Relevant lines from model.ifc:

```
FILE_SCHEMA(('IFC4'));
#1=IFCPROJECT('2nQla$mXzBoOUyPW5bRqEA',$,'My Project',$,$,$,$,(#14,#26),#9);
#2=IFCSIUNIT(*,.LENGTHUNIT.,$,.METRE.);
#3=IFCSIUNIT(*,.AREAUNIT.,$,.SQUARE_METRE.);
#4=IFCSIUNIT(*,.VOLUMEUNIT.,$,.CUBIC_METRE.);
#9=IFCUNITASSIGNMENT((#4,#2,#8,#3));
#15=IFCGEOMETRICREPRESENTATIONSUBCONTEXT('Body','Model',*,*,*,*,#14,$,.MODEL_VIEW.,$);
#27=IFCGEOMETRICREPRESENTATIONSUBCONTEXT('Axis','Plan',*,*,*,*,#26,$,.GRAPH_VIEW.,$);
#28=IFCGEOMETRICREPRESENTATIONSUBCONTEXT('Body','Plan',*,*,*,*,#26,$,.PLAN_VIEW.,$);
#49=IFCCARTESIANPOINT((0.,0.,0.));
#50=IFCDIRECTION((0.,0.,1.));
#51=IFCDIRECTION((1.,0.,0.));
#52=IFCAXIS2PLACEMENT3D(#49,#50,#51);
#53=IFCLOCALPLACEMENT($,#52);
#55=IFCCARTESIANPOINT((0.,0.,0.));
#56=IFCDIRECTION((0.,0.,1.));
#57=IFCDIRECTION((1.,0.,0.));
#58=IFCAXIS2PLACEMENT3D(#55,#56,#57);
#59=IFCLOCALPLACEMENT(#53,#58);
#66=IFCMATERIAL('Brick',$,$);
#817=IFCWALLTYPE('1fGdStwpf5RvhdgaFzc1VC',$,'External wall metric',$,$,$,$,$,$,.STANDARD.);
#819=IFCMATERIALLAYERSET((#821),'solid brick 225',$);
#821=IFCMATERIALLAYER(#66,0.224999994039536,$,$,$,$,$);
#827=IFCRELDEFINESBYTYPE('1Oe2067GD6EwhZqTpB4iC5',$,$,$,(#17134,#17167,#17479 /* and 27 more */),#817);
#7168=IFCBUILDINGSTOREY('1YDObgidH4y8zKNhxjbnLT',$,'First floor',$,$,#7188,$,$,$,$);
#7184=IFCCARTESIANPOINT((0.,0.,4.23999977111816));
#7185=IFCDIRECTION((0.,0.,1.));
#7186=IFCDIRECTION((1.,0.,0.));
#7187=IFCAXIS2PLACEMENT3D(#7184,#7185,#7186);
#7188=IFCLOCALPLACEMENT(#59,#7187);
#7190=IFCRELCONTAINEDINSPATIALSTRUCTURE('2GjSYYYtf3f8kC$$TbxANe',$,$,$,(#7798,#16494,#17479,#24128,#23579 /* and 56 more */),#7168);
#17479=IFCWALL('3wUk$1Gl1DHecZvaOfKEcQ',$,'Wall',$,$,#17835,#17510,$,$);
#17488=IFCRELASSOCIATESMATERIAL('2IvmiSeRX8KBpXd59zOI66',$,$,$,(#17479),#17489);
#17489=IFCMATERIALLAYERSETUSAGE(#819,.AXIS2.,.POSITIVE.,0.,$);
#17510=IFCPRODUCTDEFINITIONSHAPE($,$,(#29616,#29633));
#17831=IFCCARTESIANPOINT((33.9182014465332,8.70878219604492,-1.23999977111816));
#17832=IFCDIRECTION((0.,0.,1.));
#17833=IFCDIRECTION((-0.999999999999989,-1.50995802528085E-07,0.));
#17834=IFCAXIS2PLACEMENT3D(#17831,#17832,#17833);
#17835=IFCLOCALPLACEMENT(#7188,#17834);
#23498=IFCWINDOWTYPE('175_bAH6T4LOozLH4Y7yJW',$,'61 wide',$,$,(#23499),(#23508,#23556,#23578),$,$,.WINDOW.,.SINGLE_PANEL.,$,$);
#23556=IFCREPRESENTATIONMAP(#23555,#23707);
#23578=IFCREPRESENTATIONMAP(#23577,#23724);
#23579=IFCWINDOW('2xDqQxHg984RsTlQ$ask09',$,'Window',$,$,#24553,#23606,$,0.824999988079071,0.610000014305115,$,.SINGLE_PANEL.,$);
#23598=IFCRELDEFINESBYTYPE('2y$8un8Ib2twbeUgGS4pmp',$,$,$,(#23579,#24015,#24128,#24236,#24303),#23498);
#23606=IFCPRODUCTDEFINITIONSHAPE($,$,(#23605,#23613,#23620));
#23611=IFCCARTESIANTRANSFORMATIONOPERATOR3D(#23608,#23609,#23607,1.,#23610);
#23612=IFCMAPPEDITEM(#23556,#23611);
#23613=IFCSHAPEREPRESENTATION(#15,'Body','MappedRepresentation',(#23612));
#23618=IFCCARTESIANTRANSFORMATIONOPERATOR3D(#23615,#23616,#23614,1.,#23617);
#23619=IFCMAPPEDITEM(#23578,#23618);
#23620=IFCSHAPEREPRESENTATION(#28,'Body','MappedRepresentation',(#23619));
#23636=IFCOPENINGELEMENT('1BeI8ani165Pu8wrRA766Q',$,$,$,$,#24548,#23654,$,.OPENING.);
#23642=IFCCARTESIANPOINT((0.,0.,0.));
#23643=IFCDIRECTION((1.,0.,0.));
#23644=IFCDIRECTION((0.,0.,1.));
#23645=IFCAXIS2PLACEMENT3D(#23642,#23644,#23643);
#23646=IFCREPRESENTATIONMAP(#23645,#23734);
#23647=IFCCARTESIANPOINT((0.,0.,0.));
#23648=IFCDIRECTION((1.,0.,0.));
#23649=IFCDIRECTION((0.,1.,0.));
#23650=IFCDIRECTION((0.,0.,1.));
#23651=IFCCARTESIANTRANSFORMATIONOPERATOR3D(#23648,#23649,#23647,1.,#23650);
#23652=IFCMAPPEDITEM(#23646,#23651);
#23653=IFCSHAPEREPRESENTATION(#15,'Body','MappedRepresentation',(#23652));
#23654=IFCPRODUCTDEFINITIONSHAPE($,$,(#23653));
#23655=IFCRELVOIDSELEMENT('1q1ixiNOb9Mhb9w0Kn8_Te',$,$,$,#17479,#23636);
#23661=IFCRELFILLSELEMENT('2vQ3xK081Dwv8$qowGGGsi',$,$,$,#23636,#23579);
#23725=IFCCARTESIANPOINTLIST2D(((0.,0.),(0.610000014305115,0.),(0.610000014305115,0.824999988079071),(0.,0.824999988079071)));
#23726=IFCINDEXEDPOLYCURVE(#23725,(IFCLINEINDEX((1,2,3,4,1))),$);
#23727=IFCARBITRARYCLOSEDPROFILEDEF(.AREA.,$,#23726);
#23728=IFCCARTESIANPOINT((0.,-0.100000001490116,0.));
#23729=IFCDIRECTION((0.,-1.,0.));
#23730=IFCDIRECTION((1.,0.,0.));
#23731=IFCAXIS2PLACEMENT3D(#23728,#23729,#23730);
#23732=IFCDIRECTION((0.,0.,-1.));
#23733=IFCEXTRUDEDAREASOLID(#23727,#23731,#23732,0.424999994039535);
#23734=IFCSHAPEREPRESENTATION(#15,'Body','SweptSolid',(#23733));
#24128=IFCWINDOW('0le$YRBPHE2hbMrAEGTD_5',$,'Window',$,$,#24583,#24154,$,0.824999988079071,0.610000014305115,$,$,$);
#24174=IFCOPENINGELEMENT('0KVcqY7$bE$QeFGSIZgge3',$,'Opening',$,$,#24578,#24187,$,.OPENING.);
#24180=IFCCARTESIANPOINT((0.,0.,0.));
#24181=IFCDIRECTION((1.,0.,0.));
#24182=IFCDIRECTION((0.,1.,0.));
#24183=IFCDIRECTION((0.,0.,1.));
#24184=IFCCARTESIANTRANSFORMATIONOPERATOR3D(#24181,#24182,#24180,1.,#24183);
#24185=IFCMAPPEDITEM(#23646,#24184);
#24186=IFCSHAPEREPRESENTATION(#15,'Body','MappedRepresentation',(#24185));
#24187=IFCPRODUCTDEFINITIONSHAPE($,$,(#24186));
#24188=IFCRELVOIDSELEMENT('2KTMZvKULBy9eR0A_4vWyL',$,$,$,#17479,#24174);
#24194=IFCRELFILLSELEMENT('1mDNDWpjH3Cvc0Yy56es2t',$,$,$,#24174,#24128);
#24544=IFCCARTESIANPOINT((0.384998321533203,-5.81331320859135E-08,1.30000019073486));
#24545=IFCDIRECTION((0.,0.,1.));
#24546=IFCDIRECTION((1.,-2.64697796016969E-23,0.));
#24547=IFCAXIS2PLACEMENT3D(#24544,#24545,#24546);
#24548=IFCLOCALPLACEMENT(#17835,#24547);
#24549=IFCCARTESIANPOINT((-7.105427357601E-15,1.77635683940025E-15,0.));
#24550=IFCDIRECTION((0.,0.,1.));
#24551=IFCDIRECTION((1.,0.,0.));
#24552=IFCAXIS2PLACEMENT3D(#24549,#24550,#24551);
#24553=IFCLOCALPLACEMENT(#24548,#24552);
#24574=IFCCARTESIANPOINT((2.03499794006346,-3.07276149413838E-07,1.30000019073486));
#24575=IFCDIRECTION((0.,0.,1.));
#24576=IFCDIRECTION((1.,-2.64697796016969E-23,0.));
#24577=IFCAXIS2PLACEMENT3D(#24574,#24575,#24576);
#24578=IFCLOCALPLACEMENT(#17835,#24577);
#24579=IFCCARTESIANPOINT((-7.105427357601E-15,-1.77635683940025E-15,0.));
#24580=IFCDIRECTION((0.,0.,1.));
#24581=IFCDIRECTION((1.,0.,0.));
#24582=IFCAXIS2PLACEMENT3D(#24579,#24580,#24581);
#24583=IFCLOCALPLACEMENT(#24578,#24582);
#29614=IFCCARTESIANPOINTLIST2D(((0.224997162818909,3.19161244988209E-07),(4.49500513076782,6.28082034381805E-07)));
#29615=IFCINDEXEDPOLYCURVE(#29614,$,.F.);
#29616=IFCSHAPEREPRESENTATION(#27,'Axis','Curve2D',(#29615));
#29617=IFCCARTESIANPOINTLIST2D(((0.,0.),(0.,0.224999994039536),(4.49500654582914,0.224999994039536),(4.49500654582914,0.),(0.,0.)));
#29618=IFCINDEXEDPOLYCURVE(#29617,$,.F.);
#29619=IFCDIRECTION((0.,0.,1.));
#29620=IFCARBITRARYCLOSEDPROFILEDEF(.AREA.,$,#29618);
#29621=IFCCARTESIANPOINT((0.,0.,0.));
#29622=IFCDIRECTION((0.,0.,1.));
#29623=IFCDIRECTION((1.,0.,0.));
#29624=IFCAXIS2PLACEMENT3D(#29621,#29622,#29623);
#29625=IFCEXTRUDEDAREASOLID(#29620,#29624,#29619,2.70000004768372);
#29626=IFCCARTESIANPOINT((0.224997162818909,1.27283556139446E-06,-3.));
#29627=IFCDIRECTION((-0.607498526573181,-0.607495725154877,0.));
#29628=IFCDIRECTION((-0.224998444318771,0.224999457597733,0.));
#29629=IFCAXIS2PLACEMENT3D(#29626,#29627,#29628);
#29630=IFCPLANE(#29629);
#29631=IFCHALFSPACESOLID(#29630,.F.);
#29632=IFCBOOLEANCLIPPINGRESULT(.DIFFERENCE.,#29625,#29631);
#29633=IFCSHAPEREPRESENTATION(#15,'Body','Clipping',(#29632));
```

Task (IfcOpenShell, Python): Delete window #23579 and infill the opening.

```python
import ifcopenshell
import ifcopenshell.api.feature
import ifcopenshell.api.root
import ifcopenshell.geom
import ifcopenshell.util.shape

model = ifcopenshell.open("model.ifc")
settings = ifcopenshell.geom.settings()


def volume(element):
    """Net volume in cubic metres, openings subtracted."""
    shape = ifcopenshell.geom.create_shape(settings, element)
    return ifcopenshell.util.shape.get_volume(shape.geometry)


window = model.by_guid("2xDqQxHg984RsTlQ$ask09")
opening = window.FillsVoids[0].RelatingOpeningElement
wall = opening.VoidsElements[0].RelatingBuildingElement
before = volume(wall)

ifcopenshell.api.root.remove_product(model, product=window)
ifcopenshell.api.feature.remove_feature(model, feature=opening)

after = volume(wall)

print(f"wall volume {before:.3f} -> {after:.3f} m3")

model.write("model_edited.ifc")
```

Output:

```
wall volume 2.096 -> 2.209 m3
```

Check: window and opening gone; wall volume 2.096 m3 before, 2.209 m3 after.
